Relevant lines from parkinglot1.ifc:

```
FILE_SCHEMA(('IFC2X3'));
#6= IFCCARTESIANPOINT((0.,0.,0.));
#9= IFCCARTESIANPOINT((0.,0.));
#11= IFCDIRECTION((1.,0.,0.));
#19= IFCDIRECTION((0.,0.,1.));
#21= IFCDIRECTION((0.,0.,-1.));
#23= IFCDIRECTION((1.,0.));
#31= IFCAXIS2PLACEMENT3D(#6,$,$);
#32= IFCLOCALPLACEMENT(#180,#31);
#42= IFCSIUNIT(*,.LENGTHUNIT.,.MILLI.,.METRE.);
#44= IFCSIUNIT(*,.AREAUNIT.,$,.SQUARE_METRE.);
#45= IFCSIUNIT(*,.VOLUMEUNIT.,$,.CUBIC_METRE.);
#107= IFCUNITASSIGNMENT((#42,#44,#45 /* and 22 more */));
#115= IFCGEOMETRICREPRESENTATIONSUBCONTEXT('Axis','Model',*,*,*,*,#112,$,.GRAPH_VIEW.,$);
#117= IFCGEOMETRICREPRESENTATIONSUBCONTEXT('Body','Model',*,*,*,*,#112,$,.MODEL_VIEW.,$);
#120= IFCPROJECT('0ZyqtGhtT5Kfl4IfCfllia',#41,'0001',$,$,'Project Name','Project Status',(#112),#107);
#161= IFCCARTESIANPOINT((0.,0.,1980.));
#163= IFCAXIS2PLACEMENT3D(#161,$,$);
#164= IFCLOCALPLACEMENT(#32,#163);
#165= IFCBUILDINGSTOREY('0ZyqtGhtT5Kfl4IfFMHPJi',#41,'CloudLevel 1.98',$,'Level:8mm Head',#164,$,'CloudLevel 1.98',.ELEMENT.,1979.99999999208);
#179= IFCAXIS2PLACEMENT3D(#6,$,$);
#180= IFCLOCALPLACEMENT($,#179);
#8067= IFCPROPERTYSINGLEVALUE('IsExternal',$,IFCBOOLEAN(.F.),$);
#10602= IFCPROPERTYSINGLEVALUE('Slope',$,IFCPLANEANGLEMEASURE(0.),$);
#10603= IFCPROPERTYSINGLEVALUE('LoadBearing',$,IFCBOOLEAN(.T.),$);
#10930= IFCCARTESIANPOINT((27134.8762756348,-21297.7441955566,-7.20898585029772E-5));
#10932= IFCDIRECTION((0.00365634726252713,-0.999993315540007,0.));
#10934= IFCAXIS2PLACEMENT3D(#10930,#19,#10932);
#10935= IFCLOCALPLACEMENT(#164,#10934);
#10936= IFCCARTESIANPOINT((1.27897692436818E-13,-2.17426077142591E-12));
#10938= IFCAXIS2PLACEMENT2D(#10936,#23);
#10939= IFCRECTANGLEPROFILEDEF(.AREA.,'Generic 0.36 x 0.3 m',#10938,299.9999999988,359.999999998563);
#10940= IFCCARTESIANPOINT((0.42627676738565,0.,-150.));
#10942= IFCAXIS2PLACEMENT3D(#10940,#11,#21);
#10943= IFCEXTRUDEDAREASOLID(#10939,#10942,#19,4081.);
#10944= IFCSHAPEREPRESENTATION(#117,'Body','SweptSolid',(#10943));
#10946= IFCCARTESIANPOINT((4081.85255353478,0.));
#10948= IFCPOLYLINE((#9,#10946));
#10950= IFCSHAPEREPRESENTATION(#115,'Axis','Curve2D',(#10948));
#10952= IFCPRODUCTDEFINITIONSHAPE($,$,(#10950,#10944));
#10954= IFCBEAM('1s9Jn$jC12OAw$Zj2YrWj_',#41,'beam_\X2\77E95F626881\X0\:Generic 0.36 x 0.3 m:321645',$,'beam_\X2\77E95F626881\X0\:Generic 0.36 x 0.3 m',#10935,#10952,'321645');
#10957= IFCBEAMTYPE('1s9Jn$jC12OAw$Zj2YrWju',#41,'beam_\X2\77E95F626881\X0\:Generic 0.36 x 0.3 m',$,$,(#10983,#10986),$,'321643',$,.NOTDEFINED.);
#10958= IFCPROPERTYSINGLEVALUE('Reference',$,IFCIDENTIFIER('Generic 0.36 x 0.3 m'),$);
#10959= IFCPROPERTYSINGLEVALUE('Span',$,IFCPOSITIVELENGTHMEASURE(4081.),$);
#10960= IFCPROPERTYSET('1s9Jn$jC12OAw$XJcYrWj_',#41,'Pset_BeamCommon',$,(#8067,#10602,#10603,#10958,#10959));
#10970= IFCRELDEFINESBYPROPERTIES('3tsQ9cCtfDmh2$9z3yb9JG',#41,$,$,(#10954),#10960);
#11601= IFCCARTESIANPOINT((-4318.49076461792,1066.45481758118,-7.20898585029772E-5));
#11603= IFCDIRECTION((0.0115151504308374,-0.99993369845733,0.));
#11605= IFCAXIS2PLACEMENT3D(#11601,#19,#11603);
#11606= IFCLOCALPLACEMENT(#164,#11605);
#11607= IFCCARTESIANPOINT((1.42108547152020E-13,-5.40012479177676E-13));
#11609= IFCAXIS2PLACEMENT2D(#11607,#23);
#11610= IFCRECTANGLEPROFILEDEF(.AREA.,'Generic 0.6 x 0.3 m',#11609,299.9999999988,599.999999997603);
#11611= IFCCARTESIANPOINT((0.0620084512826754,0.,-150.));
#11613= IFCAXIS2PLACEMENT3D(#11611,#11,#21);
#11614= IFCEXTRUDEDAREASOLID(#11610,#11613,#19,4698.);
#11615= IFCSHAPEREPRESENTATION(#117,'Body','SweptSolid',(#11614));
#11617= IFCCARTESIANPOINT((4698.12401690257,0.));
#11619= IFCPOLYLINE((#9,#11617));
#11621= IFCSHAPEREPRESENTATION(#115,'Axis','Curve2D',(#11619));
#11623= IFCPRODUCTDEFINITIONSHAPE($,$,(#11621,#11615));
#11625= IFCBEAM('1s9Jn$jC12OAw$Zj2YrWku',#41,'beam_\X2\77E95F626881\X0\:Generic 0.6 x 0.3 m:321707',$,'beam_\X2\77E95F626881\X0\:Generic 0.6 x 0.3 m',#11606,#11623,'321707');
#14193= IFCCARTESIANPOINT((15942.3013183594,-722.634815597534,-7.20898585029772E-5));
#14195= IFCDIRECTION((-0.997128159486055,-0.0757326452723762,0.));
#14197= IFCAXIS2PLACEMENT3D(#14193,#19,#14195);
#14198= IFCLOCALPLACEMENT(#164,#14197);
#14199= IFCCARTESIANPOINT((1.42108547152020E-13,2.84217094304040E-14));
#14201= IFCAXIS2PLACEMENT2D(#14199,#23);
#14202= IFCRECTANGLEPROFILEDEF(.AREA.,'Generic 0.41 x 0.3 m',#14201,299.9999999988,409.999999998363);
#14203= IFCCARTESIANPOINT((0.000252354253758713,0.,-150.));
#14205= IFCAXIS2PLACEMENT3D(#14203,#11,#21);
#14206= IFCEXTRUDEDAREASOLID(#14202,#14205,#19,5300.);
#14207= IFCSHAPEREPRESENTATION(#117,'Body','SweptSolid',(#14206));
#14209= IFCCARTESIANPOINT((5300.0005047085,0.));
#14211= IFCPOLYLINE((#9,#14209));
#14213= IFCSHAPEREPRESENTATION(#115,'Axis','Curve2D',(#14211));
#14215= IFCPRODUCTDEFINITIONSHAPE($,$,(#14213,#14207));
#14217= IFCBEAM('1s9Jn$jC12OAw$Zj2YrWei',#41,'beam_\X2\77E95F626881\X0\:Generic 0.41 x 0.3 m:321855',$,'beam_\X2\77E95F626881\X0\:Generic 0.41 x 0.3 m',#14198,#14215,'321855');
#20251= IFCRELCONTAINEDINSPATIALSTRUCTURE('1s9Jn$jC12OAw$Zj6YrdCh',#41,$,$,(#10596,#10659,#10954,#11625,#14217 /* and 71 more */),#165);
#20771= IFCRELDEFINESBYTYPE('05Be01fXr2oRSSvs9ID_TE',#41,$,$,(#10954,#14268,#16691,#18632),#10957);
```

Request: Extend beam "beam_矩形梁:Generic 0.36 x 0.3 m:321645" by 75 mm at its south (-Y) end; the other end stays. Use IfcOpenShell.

```python
import numpy as np
import ifcopenshell
import ifcopenshell.api.pset
import ifcopenshell.util.element
import ifcopenshell.util.representation
import ifcopenshell.util.unit

model = ifcopenshell.open("parkinglot1.ifc")
unit_scale = ifcopenshell.util.unit.calculate_unit_scale(model)

member = model.by_guid("1s9Jn$jC12OAw$Zj2YrWj_")
change = 0.075 / unit_scale

# The extrusion runs towards the end named, so only its depth changes.
body = ifcopenshell.util.representation.get_representation(member, "Model", "Body")
solid = body.Items[0]
old_length = solid.Depth
solid.Depth += change

# Move the axis end point with it.
axis = next(r for r in member.Representation.Representations if r.RepresentationIdentifier == "Axis").Items[0]
start, end = (np.array(p.Coordinates) for p in axis.Points)
end = end + (end - start) / np.linalg.norm(end - start) * change
point = model.createIfcCartesianPoint(end.tolist())
axis.Points = [axis.Points[0], point]

# Update the stored length and volume.
pset = model.by_id(ifcopenshell.util.element.get_pset(member, "Pset_BeamCommon", should_inherit=False)["id"])
ifcopenshell.api.pset.edit_pset(model, pset=pset, properties={
    "Span": model.create_entity("IfcPositiveLengthMeasure", solid.Depth),
})

print(f"length {old_length:g} -> {solid.Depth:g}")

model.write("parkinglot1-out.ifc")
```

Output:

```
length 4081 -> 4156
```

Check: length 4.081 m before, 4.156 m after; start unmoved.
